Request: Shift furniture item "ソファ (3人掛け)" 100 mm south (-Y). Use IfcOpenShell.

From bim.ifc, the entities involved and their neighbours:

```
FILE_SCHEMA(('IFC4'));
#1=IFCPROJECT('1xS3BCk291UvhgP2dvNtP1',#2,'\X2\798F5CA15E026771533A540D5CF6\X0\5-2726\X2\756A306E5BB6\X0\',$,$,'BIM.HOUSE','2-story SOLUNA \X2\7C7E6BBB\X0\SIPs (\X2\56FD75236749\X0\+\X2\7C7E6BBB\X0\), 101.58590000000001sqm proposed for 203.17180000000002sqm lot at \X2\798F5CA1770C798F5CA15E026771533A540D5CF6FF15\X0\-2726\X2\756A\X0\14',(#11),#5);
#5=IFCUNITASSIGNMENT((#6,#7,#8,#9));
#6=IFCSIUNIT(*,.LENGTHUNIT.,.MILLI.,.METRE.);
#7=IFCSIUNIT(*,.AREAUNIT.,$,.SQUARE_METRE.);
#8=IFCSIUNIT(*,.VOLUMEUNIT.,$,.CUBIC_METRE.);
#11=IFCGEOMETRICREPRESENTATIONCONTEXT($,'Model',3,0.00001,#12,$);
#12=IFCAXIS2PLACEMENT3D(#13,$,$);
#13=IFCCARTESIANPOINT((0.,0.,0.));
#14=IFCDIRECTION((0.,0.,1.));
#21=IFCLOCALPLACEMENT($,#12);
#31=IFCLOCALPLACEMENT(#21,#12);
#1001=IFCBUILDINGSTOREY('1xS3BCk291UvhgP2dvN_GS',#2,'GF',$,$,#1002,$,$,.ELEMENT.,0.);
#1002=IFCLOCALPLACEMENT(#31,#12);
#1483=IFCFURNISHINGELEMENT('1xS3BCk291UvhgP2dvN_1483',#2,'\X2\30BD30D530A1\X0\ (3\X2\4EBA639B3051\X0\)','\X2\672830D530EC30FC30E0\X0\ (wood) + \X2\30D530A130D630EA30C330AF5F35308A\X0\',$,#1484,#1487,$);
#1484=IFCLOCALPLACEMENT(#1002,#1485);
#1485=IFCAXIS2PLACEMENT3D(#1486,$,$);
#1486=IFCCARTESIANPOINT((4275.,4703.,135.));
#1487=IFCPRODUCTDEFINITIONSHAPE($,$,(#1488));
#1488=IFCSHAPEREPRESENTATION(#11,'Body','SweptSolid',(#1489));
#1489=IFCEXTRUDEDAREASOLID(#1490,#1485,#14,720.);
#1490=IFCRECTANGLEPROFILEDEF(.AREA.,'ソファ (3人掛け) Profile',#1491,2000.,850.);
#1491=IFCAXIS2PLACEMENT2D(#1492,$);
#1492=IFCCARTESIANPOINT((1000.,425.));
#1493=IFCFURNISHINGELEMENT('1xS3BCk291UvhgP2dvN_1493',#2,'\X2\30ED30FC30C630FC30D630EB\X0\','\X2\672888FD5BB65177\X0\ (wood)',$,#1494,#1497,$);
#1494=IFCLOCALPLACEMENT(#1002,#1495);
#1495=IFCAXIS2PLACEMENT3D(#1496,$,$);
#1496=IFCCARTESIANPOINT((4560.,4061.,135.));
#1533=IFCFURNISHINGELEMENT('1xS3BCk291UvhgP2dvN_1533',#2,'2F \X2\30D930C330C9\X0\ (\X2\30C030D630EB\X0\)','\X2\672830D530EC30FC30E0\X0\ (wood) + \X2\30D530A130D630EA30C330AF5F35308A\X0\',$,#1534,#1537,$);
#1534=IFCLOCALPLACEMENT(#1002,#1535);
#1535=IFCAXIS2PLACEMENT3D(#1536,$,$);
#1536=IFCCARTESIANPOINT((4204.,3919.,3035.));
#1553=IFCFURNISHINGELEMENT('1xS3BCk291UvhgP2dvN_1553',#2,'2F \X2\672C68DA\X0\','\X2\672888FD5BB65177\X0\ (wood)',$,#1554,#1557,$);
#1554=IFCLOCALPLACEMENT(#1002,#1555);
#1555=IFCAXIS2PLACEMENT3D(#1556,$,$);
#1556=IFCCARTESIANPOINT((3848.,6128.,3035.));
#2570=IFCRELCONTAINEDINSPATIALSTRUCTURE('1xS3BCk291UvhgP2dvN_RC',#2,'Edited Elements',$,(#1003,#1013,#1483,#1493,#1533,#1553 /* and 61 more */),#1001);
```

```python
import ifcopenshell
import ifcopenshell.api.geometry
import ifcopenshell.util.placement
import ifcopenshell.util.unit

model = ifcopenshell.open("bim.ifc")
unit_scale = ifcopenshell.util.unit.calculate_unit_scale(model)

item = model.by_id(1483)
matrix = ifcopenshell.util.placement.get_local_placement(item.ObjectPlacement)
matrix[1, 3] -= 0.1 / unit_scale
ifcopenshell.api.geometry.edit_object_placement(model, product=item, matrix=matrix, is_si=False)

print(ifcopenshell.util.placement.get_local_placement(item.ObjectPlacement).round(3) + 0.0)

model.write("bim_edited.ifc")
```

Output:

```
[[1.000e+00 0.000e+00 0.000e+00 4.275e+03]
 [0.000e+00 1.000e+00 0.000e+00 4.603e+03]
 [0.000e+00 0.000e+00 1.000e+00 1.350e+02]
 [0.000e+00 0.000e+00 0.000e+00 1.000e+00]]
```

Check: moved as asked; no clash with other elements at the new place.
